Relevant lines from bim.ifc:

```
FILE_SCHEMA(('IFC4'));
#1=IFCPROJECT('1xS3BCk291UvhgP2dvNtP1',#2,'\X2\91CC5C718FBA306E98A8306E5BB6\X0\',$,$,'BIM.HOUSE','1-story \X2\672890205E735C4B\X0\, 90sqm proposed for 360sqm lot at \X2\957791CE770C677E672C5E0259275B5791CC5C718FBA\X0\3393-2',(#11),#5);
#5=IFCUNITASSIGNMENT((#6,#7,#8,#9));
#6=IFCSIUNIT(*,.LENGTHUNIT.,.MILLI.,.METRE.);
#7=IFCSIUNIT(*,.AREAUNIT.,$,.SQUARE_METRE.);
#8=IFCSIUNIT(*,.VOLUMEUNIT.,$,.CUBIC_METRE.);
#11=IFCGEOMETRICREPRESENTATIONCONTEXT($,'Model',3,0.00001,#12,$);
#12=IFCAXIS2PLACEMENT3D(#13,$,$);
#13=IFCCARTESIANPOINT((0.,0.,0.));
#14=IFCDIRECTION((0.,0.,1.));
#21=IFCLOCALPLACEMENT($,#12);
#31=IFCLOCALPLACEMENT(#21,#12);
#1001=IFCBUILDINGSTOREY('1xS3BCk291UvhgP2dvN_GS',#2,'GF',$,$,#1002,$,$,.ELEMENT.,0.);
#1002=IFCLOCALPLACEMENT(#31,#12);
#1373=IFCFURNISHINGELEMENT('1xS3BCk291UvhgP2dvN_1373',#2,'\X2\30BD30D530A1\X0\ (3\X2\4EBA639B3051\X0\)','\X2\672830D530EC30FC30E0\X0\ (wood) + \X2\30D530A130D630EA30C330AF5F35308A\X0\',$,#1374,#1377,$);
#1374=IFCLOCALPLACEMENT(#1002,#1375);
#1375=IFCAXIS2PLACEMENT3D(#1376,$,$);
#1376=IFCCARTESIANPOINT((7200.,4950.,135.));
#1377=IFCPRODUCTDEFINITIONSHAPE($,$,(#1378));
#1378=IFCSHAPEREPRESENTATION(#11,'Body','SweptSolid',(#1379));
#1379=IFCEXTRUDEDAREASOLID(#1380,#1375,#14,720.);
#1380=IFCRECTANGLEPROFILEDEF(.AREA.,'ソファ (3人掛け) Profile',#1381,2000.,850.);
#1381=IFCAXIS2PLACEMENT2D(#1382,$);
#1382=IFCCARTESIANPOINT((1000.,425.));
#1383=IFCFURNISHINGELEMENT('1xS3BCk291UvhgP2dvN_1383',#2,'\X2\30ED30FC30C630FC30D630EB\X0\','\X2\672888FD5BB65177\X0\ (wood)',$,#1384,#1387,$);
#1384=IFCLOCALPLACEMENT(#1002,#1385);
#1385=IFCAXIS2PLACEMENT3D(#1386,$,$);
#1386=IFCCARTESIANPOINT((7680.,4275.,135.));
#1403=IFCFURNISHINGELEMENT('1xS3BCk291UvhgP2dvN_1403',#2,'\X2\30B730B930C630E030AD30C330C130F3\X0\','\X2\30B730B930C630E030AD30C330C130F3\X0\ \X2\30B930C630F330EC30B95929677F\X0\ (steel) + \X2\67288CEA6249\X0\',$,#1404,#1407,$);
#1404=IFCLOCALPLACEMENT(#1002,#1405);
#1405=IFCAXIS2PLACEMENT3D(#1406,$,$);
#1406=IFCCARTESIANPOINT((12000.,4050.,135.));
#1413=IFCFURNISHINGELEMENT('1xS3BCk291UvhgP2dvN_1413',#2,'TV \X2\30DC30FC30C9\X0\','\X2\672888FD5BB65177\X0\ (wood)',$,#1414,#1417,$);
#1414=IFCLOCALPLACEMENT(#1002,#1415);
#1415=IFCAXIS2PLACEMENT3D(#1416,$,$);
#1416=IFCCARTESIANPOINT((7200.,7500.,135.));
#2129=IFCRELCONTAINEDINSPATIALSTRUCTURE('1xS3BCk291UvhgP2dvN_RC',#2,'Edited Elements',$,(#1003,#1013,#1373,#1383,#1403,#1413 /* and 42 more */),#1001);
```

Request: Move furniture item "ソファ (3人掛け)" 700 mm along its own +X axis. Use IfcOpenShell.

```python
import ifcopenshell
import ifcopenshell.api.geometry
import ifcopenshell.util.placement
import ifcopenshell.util.unit

model = ifcopenshell.open("bim.ifc")
unit_scale = ifcopenshell.util.unit.calculate_unit_scale(model)

item = model.by_id(1373)
matrix = ifcopenshell.util.placement.get_local_placement(item.ObjectPlacement)
matrix[:3, 3] += matrix[:3, 0] * 0.7 / unit_scale
ifcopenshell.api.geometry.edit_object_placement(model, product=item, matrix=matrix, is_si=False)

print(ifcopenshell.util.placement.get_local_placement(item.ObjectPlacement).round(3) + 0.0)

model.write("bim_v2.ifc")
```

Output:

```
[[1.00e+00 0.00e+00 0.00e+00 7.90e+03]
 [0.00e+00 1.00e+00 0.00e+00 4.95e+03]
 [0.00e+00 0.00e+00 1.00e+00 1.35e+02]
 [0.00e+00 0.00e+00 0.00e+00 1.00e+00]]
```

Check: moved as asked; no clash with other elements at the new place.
